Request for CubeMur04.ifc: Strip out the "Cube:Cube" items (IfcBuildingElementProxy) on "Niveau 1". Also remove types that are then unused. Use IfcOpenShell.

First a look at what the model holds.

```python
import ifcopenshell
import ifcopenshell.util.element

model = ifcopenshell.open("CubeMur04.ifc")
print(model.schema)
storey = next(s for s in model.by_type("IfcBuildingStorey") if s.Name == "Niveau 1")
proxies = [e for e in ifcopenshell.util.element.get_decomposition(storey) if e.is_a("IfcBuildingElementProxy")]
seen = {}
for e in proxies:
    element_type = ifcopenshell.util.element.get_type(e)
    name = element_type.Name if element_type not in (None, e) else None
    seen[name] = seen.get(name, 0) + 1
for name, count in sorted(seen.items(), key=str):
    print(count, "x", name)
```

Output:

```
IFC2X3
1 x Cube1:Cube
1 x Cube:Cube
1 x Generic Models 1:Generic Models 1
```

```python
import ifcopenshell
import ifcopenshell.api.root
import ifcopenshell.util.element

model = ifcopenshell.open("CubeMur04.ifc")

storey = next(s for s in model.by_type("IfcBuildingStorey") if s.Name == "Niveau 1")
proxies = [e for e in ifcopenshell.util.element.get_decomposition(storey) if e.is_a("IfcBuildingElementProxy")]
targets = [e for e in proxies if (t := ifcopenshell.util.element.get_type(e)) not in (None, e) and t.Name == "Cube:Cube"]
types = {ifcopenshell.util.element.get_type(e) for e in targets} - {None, *targets}

for e in targets:
    ifcopenshell.api.root.remove_product(model, product=e)
print(len(targets), "removed")

unused = [t for t in types if not ifcopenshell.util.element.get_types(t)]
for t in unused:
    ifcopenshell.api.root.remove_product(model, product=t)
print(len(unused), "unused types removed")

model.write("CubeMur04_edited.ifc")
```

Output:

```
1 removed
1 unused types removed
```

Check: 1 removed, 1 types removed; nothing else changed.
